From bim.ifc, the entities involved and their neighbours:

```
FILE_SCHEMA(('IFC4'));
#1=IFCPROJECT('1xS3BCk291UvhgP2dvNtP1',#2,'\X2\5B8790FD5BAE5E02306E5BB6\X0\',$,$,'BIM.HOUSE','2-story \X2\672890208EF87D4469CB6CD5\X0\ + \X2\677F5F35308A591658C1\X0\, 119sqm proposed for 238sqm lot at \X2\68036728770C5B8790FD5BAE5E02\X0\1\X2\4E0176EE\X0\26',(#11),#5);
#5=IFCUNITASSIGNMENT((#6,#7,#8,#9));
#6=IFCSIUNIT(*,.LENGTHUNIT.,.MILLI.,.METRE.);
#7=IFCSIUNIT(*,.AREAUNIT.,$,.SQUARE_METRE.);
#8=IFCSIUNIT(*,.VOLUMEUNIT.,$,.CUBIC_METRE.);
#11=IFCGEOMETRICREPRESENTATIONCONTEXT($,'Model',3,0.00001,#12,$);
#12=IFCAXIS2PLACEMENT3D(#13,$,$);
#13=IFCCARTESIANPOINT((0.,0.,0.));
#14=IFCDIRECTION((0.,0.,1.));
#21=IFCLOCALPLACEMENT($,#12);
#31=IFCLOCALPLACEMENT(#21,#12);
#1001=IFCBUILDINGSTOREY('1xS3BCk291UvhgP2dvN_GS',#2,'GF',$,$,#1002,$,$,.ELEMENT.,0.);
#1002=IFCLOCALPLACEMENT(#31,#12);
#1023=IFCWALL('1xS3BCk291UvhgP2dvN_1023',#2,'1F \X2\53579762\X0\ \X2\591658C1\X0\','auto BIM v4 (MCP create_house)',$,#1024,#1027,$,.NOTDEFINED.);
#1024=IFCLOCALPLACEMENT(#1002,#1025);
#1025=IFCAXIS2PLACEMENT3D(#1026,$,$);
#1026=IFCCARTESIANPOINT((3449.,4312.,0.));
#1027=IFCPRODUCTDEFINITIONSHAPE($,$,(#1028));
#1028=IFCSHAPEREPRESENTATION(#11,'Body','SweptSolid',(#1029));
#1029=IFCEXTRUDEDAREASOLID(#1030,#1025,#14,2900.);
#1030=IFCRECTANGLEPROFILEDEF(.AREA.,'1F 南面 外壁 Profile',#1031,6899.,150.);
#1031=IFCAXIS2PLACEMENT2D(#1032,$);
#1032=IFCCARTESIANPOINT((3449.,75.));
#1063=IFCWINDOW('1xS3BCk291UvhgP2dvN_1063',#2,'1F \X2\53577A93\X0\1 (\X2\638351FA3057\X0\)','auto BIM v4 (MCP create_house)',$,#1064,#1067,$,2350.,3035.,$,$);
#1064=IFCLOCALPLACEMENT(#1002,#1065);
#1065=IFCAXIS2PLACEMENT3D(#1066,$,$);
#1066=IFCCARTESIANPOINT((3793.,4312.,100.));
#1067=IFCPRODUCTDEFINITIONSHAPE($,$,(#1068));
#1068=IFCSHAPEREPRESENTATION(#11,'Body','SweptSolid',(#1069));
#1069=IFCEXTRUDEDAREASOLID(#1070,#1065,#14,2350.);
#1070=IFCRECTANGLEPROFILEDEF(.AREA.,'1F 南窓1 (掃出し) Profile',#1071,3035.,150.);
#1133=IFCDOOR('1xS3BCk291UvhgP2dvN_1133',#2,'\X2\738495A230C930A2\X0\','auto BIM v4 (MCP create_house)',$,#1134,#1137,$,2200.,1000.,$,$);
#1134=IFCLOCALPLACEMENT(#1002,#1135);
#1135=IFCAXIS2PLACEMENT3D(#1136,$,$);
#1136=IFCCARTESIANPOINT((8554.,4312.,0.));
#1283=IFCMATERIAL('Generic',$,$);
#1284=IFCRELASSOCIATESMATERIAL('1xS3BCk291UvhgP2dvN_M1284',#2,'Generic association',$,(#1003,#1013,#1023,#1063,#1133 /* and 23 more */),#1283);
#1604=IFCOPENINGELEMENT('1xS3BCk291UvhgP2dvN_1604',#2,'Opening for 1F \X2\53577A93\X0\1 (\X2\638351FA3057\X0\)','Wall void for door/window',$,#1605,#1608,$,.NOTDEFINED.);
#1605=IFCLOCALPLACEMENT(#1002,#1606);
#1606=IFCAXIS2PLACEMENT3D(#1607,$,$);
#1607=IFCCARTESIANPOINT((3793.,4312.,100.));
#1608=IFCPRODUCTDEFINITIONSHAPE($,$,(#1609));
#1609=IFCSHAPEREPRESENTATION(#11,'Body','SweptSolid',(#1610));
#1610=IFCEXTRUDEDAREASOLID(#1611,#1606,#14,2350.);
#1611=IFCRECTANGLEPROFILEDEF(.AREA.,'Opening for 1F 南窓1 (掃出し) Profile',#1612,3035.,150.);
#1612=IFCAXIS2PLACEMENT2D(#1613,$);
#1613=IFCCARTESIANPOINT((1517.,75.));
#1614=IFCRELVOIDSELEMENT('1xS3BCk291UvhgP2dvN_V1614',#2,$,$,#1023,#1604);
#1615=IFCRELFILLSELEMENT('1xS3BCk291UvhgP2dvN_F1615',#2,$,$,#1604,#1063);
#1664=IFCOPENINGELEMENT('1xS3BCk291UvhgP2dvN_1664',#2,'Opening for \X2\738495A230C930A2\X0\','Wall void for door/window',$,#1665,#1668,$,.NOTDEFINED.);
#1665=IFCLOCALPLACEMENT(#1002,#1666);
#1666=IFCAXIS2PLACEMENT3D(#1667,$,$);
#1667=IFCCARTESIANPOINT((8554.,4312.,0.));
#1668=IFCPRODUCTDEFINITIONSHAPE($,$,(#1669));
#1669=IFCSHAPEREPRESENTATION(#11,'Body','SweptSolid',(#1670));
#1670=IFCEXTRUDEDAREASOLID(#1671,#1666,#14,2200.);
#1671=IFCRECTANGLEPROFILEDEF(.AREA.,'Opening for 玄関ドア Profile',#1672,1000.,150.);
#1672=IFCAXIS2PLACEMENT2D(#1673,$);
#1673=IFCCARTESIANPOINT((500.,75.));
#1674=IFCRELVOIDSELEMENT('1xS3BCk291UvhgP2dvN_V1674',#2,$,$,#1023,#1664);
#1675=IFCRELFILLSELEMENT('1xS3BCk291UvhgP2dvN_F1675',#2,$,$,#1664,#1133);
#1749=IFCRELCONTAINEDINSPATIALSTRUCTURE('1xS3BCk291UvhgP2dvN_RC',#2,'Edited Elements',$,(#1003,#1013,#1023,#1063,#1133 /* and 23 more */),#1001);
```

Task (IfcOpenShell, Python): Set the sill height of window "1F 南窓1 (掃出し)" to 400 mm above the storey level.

```python
import numpy as np
import ifcopenshell
import ifcopenshell.api.geometry
import ifcopenshell.geom
import ifcopenshell.util.element
import ifcopenshell.util.placement
import ifcopenshell.util.shape
import ifcopenshell.util.unit

model = ifcopenshell.open("bim.ifc")
unit_scale = ifcopenshell.util.unit.calculate_unit_scale(model)

window = model.by_guid("1xS3BCk291UvhgP2dvN_1063")
opening = window.FillsVoids[0].RelatingOpeningElement
storey = ifcopenshell.util.element.get_container(window, ifc_class="IfcBuildingStorey")
level = ifcopenshell.util.placement.get_local_placement(storey.ObjectPlacement)[2, 3]

# The opening's origin need not be at the sill, so measure its lowest point.
shape = ifcopenshell.geom.create_shape(ifcopenshell.geom.settings(), opening)
bottom = ifcopenshell.util.shape.get_shape_bottom_elevation(shape, shape.geometry) / unit_scale
dz = level + 400.0 - bottom

shift = np.array([0.0, 0.0, dz])
# The window is not placed relative to its opening, so move both.
for product in (opening, window):
    matrix = ifcopenshell.util.placement.get_local_placement(product.ObjectPlacement)
    matrix[:3, 3] += shift
    ifcopenshell.api.geometry.edit_object_placement(model, product=product, matrix=matrix, is_si=False)

print(f"moved by {dz * unit_scale:+.3f} m")

model.write("bim_updated.ifc")
```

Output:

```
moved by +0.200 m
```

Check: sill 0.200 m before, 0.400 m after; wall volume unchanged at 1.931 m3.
